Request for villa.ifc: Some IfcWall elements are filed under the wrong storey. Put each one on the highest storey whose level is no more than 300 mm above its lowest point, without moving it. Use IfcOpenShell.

First a look at what the model holds.

```python
import ifcopenshell
import ifcopenshell.util.element
import ifcopenshell.util.placement

model = ifcopenshell.open("villa.ifc")
print(model.schema)
for storey in model.by_type("IfcBuildingStorey"):
    level = ifcopenshell.util.placement.get_storey_elevation(storey)
    count = sum(e.is_a("IfcWall") for e in ifcopenshell.util.element.get_contained(storey))
    print(storey.id(), storey.Name, round(level, 3), count, sep=" | ")
```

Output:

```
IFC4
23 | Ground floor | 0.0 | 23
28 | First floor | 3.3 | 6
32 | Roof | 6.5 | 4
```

```python
import ifcopenshell
import ifcopenshell.api.spatial
import ifcopenshell.geom
import ifcopenshell.util.element
import ifcopenshell.util.placement
import ifcopenshell.util.shape
import ifcopenshell.util.unit

model = ifcopenshell.open("villa.ifc")
unit_scale = ifcopenshell.util.unit.calculate_unit_scale(model)
settings = ifcopenshell.geom.settings()

levels = sorted(
    ((ifcopenshell.util.placement.get_storey_elevation(s) * unit_scale, s) for s in model.by_type("IfcBuildingStorey")),
    key=lambda pair: pair[0],
)

for e in model.by_type("IfcWall"):
    current = e.ContainedInStructure[0].RelatingStructure if e.ContainedInStructure else None
    if current is None or not current.is_a("IfcBuildingStorey"):
        continue
    shape = ifcopenshell.geom.create_shape(settings, e)
    bottom = ifcopenshell.util.shape.get_shape_bottom_elevation(shape, shape.geometry)
    below = [s for level, s in levels if level <= bottom + 0.3]
    storey = below[-1] if below else levels[0][1]
    if storey != current:
        # assign_container keeps the world position.
        ifcopenshell.api.spatial.assign_container(model, products=[e], relating_structure=storey)
        print(e.id(), current.Name, "->", storey.Name)

model.write("villa_v2.ifc")
```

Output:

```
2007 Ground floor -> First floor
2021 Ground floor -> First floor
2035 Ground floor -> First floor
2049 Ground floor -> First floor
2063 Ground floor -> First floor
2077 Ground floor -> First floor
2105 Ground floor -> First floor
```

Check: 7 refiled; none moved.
